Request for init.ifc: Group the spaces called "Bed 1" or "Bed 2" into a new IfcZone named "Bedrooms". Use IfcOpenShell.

First a look at what the model holds.

```python
import ifcopenshell

model = ifcopenshell.open("init.ifc")
print(model.schema)
seen = {}
for space in model.by_type("IfcSpace"):
    seen[space.Name] = seen.get(space.Name, 0) + 1
for name, count in sorted(seen.items(), key=str):
    print(count, "x", name)
print("zones:", [z.Name for z in model.by_type("IfcZone")][:20])
```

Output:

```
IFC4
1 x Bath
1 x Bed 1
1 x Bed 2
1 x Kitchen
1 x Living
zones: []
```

```python
import ifcopenshell
import ifcopenshell.api.group
import ifcopenshell.api.root

model = ifcopenshell.open("init.ifc")

names = {"Bed 1", "Bed 2"}
spaces = [s for s in model.by_type("IfcSpace") if s.Name in names]

zone = ifcopenshell.api.root.create_entity(model, ifc_class="IfcZone", name="Bedrooms")
ifcopenshell.api.group.assign_group(model, products=spaces, group=zone)
print(len(spaces), "spaces in", zone.Name)

model.write("init_edited.ifc")
```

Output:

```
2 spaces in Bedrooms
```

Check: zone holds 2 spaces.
